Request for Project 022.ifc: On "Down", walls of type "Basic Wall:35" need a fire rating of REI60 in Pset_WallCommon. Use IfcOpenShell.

First a look at what the model holds.

```python
import ifcopenshell
import ifcopenshell.util.element

model = ifcopenshell.open("Project 022.ifc")
print(model.schema)
storey = next(s for s in model.by_type("IfcBuildingStorey") if s.Name == "Down")
walls = [e for e in ifcopenshell.util.element.get_decomposition(storey) if e.is_a("IfcWall")]
seen = {}
for e in walls:
    element_type = ifcopenshell.util.element.get_type(e)
    key = (element_type.Name if element_type != e and element_type else None, ifcopenshell.util.element.get_pset(e, "Pset_WallCommon", "FireRating"))
    seen[key] = seen.get(key, 0) + 1
for (name, value), count in sorted(seen.items(), key=str):
    print(count, "x", name, "|", value)
```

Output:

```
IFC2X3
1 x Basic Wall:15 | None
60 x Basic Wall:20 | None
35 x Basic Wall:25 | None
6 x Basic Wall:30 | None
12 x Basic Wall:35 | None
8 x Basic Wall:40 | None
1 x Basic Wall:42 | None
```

```python
import ifcopenshell
import ifcopenshell.api.pset
import ifcopenshell.util.element

model = ifcopenshell.open("Project 022.ifc")

storey = next(s for s in model.by_type("IfcBuildingStorey") if s.Name == "Down")
walls = [e for e in ifcopenshell.util.element.get_decomposition(storey) if e.is_a("IfcWall")]

count = 0
for e in walls:
    element_type = ifcopenshell.util.element.get_type(e)
    if element_type in (None, e) or element_type.Name != "Basic Wall:35":
        continue
    # add_pset returns the element's existing set when there is one.
    pset = ifcopenshell.api.pset.add_pset(model, product=e, name="Pset_WallCommon")
    ifcopenshell.api.pset.edit_pset(model, pset=pset, properties={"FireRating": "REI60"})
    count += 1

print(count, "walls updated")

model.write("Project 022_updated.ifc")
```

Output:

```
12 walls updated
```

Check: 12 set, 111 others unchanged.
